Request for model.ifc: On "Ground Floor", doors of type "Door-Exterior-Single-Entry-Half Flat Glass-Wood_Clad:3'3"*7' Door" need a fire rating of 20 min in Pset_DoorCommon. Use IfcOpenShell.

First a look at what the model holds.

```python
import ifcopenshell
import ifcopenshell.util.element

model = ifcopenshell.open("model.ifc")
print(model.schema)
storey = next(s for s in model.by_type("IfcBuildingStorey") if s.Name == "Ground Floor")
doors = [e for e in ifcopenshell.util.element.get_decomposition(storey) if e.is_a("IfcDoor")]
seen = {}
for e in doors:
    element_type = ifcopenshell.util.element.get_type(e)
    key = (element_type.Name if element_type != e and element_type else None, ifcopenshell.util.element.get_pset(e, "Pset_DoorCommon", "FireRating"))
    seen[key] = seen.get(key, 0) + 1
for (name, value), count in sorted(seen.items(), key=str):
    print(count, "x", name, "|", value)
```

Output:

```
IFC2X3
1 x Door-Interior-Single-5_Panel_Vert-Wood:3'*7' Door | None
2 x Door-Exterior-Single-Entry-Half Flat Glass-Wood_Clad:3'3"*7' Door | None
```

```python
import ifcopenshell
import ifcopenshell.api.pset
import ifcopenshell.util.element

model = ifcopenshell.open("model.ifc")

storey = next(s for s in model.by_type("IfcBuildingStorey") if s.Name == "Ground Floor")
doors = [e for e in ifcopenshell.util.element.get_decomposition(storey) if e.is_a("IfcDoor")]

count = 0
for e in doors:
    element_type = ifcopenshell.util.element.get_type(e)
    if element_type in (None, e) or element_type.Name != 'Door-Exterior-Single-Entry-Half Flat Glass-Wood_Clad:3\'3"*7\' Door':
        continue
    # add_pset returns the element's existing set when there is one.
    pset = ifcopenshell.api.pset.add_pset(model, product=e, name="Pset_DoorCommon")
    ifcopenshell.api.pset.edit_pset(model, pset=pset, properties={"FireRating": "20 min"})
    count += 1

print(count, "doors updated")

model.write("model-out.ifc")
```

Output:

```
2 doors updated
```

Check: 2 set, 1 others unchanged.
